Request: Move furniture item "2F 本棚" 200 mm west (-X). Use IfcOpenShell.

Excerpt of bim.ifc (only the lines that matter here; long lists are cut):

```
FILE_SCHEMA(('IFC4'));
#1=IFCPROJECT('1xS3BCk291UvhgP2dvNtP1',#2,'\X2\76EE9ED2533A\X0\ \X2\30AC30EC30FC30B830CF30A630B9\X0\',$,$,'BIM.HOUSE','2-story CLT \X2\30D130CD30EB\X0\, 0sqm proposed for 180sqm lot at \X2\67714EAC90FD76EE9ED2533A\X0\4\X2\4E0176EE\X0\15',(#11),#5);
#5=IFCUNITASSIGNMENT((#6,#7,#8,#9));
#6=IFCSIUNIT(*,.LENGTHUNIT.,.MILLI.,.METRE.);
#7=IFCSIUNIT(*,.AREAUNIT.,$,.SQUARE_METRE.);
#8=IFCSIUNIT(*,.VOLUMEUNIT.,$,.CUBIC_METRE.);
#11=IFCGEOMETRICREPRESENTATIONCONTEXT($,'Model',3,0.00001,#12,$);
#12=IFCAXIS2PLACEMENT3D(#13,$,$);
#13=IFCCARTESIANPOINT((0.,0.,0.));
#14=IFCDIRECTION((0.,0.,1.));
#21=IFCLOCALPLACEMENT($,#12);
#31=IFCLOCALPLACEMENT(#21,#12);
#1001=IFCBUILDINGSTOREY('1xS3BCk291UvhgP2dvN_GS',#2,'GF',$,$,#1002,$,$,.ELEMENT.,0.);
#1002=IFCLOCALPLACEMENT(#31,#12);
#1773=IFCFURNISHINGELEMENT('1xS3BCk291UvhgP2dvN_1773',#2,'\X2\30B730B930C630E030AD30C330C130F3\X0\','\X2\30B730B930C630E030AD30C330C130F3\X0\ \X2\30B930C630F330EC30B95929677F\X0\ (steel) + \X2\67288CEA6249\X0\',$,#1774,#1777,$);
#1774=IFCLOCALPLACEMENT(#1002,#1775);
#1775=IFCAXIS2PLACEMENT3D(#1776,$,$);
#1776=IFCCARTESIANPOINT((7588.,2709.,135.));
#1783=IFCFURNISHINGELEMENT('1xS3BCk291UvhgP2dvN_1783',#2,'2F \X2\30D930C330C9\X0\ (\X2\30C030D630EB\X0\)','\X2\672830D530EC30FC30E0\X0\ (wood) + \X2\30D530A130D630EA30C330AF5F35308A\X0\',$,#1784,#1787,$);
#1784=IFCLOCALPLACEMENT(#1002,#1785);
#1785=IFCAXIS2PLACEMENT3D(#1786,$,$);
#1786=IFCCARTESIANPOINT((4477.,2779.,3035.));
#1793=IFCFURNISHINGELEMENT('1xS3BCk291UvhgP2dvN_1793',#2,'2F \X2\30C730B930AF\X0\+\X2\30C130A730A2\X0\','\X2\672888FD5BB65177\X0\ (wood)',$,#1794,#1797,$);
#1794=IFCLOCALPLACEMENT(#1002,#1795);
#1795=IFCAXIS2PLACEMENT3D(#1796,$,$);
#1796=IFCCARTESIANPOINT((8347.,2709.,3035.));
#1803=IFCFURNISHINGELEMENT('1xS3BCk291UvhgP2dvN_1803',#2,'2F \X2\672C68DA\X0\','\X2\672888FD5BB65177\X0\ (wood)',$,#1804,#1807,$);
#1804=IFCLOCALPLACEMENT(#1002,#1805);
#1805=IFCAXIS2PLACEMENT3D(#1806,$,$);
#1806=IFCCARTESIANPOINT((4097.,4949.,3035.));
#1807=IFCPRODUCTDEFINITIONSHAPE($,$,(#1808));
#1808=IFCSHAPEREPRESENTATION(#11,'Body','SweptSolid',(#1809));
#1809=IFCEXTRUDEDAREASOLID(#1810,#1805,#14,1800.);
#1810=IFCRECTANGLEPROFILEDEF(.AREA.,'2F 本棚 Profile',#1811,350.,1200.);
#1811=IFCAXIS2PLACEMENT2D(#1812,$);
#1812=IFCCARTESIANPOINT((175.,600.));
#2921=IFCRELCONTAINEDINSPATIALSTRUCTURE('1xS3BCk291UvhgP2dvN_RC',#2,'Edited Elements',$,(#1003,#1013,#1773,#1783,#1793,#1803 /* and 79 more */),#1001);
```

```python
import ifcopenshell
import ifcopenshell.api.geometry
import ifcopenshell.util.placement
import ifcopenshell.util.unit

model = ifcopenshell.open("bim.ifc")
unit_scale = ifcopenshell.util.unit.calculate_unit_scale(model)

item = model.by_guid("1xS3BCk291UvhgP2dvN_1803")
matrix = ifcopenshell.util.placement.get_local_placement(item.ObjectPlacement)
matrix[0, 3] -= 0.2 / unit_scale
ifcopenshell.api.geometry.edit_object_placement(model, product=item, matrix=matrix, is_si=False)

print(ifcopenshell.util.placement.get_local_placement(item.ObjectPlacement).round(3) + 0.0)

model.write("bim_rev.ifc")
```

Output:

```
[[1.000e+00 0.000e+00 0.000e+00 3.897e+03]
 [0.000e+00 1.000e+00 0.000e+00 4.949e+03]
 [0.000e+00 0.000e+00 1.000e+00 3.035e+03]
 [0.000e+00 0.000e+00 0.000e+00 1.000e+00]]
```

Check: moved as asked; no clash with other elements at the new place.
